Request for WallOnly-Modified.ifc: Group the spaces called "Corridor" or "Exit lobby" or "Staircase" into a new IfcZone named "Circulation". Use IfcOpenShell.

First a look at what the model holds.

```python
import ifcopenshell

model = ifcopenshell.open("WallOnly-Modified.ifc")
print(model.schema)
seen = {}
for space in model.by_type("IfcSpace"):
    seen[space.LongName] = seen.get(space.LongName, 0) + 1
for name, count in sorted(seen.items(), key=str):
    print(count, "x", name)
print("zones:", [z.Name for z in model.by_type("IfcZone")][:20])
```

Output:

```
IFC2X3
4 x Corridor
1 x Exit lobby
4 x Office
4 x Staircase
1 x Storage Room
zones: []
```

```python
import ifcopenshell
import ifcopenshell.api.group
import ifcopenshell.api.root

model = ifcopenshell.open("WallOnly-Modified.ifc")

names = {"Corridor", "Exit lobby", "Staircase"}
spaces = [s for s in model.by_type("IfcSpace") if s.LongName in names]

zone = ifcopenshell.api.root.create_entity(model, ifc_class="IfcZone", name="Circulation")
ifcopenshell.api.group.assign_group(model, products=spaces, group=zone)
print(len(spaces), "spaces in", zone.Name)

model.write("WallOnly-Modified_rev.ifc")
```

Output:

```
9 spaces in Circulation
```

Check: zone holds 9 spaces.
